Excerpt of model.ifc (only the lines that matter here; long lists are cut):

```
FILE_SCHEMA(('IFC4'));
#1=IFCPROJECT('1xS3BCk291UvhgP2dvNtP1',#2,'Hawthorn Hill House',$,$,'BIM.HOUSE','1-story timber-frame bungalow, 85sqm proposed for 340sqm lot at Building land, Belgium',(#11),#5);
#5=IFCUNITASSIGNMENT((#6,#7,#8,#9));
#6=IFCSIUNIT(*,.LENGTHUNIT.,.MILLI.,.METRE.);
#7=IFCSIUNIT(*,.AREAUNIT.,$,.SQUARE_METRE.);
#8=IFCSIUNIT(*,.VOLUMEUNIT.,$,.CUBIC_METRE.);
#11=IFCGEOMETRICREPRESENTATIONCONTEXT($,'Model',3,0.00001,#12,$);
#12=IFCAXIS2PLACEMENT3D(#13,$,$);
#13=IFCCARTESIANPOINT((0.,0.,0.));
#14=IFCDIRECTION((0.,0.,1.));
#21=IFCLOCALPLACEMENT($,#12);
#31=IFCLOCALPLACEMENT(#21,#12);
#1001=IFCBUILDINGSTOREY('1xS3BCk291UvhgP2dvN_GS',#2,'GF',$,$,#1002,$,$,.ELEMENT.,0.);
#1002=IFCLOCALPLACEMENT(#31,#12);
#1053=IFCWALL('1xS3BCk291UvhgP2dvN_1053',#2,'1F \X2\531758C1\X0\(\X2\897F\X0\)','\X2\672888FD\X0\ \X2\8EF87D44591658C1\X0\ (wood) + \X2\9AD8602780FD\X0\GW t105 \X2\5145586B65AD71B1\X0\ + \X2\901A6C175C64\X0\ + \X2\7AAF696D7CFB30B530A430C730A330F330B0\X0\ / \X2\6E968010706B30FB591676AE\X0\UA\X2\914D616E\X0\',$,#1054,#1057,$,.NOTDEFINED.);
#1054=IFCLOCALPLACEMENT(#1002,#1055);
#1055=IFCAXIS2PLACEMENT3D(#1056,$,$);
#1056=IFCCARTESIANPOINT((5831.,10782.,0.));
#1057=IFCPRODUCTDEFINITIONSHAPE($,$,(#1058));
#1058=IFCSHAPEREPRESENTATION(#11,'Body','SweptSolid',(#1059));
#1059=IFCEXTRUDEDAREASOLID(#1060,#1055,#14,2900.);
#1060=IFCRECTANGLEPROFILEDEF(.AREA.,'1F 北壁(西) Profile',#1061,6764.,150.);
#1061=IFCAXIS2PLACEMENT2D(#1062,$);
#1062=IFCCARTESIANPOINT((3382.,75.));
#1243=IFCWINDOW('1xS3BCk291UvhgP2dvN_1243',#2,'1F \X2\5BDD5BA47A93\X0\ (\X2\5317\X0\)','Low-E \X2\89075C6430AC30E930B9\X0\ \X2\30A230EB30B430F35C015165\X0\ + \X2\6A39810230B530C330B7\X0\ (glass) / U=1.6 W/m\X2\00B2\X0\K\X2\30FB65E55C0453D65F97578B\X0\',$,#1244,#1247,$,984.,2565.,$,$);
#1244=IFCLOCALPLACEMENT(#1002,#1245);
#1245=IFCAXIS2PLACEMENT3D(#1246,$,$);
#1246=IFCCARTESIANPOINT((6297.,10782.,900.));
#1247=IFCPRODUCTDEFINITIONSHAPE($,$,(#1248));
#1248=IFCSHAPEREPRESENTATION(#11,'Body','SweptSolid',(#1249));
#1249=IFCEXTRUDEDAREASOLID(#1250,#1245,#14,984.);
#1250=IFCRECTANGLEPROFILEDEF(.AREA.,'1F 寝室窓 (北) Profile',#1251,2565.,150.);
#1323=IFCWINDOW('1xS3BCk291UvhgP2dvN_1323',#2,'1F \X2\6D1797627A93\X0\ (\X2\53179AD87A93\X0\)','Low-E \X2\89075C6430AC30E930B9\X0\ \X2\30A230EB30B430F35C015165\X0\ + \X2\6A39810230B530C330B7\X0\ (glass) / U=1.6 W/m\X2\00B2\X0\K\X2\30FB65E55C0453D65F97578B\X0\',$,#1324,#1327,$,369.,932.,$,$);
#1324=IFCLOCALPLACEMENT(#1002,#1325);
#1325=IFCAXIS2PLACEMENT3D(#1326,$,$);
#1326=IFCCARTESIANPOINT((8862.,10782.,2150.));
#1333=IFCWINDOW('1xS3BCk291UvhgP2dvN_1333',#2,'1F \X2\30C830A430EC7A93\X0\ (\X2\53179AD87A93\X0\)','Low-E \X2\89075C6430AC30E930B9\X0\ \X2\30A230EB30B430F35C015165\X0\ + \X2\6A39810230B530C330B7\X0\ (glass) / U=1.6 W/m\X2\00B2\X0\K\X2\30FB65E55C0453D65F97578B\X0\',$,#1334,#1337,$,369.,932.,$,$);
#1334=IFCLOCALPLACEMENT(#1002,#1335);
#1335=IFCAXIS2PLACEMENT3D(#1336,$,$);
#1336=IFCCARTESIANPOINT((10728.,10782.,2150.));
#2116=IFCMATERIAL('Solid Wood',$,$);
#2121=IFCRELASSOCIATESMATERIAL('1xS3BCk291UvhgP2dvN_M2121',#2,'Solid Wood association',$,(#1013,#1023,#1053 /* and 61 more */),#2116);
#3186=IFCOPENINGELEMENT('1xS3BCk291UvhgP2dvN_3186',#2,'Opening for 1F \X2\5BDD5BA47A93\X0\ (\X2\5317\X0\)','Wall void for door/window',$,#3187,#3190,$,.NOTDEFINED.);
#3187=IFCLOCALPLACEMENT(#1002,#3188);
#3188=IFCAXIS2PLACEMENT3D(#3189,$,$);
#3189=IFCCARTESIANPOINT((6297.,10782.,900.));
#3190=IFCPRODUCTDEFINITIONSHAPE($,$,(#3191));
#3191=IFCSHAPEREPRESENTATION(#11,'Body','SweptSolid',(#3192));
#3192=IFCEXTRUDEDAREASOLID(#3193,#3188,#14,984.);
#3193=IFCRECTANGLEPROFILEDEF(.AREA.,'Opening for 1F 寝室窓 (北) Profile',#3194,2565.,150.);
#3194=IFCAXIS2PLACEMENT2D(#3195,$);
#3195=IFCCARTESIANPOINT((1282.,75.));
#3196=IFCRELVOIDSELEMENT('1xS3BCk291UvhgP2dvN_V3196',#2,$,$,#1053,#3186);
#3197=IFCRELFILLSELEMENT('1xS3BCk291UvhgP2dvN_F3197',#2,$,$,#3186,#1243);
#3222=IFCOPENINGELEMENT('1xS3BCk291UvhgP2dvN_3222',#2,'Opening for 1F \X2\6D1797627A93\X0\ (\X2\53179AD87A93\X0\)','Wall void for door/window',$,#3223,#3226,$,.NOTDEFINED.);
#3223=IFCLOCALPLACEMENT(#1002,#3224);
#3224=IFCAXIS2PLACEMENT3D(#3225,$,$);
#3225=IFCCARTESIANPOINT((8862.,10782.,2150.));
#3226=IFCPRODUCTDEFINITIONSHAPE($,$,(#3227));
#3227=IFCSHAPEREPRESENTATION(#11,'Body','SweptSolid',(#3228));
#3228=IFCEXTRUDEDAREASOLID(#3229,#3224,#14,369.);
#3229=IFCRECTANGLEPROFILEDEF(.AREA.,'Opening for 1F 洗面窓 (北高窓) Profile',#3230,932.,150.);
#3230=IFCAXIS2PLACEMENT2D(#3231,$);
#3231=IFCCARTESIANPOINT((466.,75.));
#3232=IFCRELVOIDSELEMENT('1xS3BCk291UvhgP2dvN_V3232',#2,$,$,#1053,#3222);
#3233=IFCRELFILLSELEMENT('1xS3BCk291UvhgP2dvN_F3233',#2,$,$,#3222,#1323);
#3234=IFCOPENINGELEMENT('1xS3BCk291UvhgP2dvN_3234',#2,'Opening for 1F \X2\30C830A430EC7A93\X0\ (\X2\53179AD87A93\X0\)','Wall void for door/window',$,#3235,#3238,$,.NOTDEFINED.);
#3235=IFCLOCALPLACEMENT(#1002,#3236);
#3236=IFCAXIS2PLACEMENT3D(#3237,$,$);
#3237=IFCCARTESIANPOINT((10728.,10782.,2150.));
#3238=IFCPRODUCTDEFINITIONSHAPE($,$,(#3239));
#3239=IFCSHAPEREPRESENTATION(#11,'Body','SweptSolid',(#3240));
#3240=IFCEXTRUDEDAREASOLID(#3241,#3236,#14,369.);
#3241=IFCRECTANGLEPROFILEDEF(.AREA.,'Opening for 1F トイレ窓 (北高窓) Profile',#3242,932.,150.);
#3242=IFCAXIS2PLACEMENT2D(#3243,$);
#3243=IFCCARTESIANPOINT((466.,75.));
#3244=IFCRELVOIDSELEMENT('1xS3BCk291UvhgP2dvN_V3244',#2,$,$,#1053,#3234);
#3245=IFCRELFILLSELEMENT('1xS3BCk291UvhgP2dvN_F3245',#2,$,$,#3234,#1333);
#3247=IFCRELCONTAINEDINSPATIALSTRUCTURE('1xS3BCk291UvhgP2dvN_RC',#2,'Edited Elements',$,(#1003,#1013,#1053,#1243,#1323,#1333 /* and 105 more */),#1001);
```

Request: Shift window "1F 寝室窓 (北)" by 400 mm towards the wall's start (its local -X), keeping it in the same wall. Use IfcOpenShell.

```python
import ifcopenshell
import ifcopenshell.api.geometry
import ifcopenshell.util.placement
import ifcopenshell.util.unit

model = ifcopenshell.open("model.ifc")
unit_scale = ifcopenshell.util.unit.calculate_unit_scale(model)

window = model.by_id(1243)
opening = window.FillsVoids[0].RelatingOpeningElement
wall = opening.VoidsElements[0].RelatingBuildingElement

wall_matrix = ifcopenshell.util.placement.get_local_placement(wall.ObjectPlacement)
shift = wall_matrix[:3, 0] * -0.4 / unit_scale
before = ifcopenshell.util.placement.get_local_placement(window.ObjectPlacement)[:3, 3].copy()

# The window is not placed relative to its opening, so move both.
for product in (opening, window):
    matrix = ifcopenshell.util.placement.get_local_placement(product.ObjectPlacement)
    matrix[:3, 3] += shift
    ifcopenshell.api.geometry.edit_object_placement(model, product=product, matrix=matrix, is_si=False)

after = ifcopenshell.util.placement.get_local_placement(window.ObjectPlacement)[:3, 3]
print("window moved by", (after - before).round(3) + 0.0)

model.write("model_v2.ifc")
```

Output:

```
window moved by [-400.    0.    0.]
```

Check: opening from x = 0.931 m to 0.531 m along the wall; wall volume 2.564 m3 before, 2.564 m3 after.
